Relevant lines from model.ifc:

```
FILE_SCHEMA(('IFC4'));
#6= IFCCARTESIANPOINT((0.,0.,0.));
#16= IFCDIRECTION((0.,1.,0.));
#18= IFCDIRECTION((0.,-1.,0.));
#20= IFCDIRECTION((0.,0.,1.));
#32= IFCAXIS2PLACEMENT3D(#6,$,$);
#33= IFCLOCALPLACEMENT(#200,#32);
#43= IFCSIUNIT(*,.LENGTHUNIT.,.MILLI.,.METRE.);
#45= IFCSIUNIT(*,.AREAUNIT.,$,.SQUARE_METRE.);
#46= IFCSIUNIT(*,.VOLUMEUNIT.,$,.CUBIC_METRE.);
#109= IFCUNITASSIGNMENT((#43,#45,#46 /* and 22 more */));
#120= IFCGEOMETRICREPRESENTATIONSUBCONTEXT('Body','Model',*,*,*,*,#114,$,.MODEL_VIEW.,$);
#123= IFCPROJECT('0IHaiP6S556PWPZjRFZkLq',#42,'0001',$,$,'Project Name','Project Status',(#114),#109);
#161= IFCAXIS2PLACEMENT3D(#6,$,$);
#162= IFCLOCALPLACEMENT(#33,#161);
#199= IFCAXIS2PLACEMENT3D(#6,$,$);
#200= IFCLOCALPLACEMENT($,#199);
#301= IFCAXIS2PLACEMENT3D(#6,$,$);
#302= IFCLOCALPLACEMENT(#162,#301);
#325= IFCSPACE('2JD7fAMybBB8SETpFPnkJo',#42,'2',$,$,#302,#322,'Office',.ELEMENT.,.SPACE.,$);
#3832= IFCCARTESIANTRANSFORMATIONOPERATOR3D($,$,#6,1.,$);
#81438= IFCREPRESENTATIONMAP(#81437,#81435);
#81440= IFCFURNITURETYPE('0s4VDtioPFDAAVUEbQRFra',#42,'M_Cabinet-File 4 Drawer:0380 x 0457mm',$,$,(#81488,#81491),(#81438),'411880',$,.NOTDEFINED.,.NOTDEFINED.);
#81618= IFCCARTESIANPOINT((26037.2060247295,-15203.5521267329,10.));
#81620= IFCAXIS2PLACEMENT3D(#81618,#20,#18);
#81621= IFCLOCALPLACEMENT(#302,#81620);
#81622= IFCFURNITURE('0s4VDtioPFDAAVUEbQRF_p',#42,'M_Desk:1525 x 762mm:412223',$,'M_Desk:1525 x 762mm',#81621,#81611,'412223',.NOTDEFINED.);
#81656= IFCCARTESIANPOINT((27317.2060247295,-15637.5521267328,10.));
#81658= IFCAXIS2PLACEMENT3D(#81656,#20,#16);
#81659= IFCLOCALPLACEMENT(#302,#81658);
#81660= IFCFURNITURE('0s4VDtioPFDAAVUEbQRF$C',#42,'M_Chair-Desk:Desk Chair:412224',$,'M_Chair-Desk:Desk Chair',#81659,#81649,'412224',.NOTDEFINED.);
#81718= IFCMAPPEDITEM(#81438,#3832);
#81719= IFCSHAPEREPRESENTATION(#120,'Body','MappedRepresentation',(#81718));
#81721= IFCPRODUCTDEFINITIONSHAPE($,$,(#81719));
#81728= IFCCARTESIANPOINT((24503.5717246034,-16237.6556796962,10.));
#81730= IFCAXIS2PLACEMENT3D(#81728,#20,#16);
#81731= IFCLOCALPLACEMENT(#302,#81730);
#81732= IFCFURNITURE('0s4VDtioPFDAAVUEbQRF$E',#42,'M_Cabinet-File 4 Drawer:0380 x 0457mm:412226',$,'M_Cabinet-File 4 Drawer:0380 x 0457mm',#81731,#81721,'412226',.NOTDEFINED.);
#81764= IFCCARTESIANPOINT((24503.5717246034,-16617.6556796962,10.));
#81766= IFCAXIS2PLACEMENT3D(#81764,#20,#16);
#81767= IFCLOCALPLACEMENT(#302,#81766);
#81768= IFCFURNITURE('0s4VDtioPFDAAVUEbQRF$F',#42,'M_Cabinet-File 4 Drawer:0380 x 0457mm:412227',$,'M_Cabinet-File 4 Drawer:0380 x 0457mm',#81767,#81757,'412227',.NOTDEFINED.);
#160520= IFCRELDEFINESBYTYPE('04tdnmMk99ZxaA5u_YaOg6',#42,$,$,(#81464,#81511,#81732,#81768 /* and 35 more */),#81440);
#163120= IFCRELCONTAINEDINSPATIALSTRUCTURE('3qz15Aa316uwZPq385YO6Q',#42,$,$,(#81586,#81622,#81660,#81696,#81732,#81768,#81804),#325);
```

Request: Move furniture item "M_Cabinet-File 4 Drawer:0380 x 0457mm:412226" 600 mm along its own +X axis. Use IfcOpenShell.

```python
import ifcopenshell
import ifcopenshell.api.geometry
import ifcopenshell.util.placement
import ifcopenshell.util.unit

model = ifcopenshell.open("model.ifc")
unit_scale = ifcopenshell.util.unit.calculate_unit_scale(model)

item = model.by_id(81732)
matrix = ifcopenshell.util.placement.get_local_placement(item.ObjectPlacement)
matrix[:3, 3] += matrix[:3, 0] * 0.6 / unit_scale
ifcopenshell.api.geometry.edit_object_placement(model, product=item, matrix=matrix, is_si=False)

print(ifcopenshell.util.placement.get_local_placement(item.ObjectPlacement).round(3) + 0.0)

model.write("model_edited.ifc")
```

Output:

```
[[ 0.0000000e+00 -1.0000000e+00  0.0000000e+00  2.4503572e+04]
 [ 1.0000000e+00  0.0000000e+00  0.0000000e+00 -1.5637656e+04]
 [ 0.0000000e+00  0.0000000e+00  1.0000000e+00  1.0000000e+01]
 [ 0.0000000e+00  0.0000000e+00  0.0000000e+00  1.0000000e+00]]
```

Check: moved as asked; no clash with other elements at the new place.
